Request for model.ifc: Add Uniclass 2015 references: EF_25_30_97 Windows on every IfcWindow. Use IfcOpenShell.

First a look at what the model holds.

```python
import ifcopenshell

model = ifcopenshell.open("model.ifc")
print(model.schema)
print("classifications:", [c.Name for c in model.by_type("IfcClassification")])
for ifc_class in ("IfcDoor", "IfcRoof", "IfcStair", "IfcWall", "IfcWindow"):
    print(ifc_class, len(model.by_type(ifc_class)))
```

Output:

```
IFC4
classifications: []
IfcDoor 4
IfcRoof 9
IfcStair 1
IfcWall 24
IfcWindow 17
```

```python
import ifcopenshell
import ifcopenshell.api.classification

model = ifcopenshell.open("model.ifc")

system = ifcopenshell.api.classification.add_classification(model, classification="Uniclass 2015")

codes = {
    "IfcWindow": ("EF_25_30_97", "Windows"),
}
for ifc_class, (code, name) in codes.items():
    products = model.by_type(ifc_class)
    ifcopenshell.api.classification.add_reference(
        model, products=products, classification=system, identification=code, name=name
    )
    print(code, len(products))

model.write("model_edited.ifc")
```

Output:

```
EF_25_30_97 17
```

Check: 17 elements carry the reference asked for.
